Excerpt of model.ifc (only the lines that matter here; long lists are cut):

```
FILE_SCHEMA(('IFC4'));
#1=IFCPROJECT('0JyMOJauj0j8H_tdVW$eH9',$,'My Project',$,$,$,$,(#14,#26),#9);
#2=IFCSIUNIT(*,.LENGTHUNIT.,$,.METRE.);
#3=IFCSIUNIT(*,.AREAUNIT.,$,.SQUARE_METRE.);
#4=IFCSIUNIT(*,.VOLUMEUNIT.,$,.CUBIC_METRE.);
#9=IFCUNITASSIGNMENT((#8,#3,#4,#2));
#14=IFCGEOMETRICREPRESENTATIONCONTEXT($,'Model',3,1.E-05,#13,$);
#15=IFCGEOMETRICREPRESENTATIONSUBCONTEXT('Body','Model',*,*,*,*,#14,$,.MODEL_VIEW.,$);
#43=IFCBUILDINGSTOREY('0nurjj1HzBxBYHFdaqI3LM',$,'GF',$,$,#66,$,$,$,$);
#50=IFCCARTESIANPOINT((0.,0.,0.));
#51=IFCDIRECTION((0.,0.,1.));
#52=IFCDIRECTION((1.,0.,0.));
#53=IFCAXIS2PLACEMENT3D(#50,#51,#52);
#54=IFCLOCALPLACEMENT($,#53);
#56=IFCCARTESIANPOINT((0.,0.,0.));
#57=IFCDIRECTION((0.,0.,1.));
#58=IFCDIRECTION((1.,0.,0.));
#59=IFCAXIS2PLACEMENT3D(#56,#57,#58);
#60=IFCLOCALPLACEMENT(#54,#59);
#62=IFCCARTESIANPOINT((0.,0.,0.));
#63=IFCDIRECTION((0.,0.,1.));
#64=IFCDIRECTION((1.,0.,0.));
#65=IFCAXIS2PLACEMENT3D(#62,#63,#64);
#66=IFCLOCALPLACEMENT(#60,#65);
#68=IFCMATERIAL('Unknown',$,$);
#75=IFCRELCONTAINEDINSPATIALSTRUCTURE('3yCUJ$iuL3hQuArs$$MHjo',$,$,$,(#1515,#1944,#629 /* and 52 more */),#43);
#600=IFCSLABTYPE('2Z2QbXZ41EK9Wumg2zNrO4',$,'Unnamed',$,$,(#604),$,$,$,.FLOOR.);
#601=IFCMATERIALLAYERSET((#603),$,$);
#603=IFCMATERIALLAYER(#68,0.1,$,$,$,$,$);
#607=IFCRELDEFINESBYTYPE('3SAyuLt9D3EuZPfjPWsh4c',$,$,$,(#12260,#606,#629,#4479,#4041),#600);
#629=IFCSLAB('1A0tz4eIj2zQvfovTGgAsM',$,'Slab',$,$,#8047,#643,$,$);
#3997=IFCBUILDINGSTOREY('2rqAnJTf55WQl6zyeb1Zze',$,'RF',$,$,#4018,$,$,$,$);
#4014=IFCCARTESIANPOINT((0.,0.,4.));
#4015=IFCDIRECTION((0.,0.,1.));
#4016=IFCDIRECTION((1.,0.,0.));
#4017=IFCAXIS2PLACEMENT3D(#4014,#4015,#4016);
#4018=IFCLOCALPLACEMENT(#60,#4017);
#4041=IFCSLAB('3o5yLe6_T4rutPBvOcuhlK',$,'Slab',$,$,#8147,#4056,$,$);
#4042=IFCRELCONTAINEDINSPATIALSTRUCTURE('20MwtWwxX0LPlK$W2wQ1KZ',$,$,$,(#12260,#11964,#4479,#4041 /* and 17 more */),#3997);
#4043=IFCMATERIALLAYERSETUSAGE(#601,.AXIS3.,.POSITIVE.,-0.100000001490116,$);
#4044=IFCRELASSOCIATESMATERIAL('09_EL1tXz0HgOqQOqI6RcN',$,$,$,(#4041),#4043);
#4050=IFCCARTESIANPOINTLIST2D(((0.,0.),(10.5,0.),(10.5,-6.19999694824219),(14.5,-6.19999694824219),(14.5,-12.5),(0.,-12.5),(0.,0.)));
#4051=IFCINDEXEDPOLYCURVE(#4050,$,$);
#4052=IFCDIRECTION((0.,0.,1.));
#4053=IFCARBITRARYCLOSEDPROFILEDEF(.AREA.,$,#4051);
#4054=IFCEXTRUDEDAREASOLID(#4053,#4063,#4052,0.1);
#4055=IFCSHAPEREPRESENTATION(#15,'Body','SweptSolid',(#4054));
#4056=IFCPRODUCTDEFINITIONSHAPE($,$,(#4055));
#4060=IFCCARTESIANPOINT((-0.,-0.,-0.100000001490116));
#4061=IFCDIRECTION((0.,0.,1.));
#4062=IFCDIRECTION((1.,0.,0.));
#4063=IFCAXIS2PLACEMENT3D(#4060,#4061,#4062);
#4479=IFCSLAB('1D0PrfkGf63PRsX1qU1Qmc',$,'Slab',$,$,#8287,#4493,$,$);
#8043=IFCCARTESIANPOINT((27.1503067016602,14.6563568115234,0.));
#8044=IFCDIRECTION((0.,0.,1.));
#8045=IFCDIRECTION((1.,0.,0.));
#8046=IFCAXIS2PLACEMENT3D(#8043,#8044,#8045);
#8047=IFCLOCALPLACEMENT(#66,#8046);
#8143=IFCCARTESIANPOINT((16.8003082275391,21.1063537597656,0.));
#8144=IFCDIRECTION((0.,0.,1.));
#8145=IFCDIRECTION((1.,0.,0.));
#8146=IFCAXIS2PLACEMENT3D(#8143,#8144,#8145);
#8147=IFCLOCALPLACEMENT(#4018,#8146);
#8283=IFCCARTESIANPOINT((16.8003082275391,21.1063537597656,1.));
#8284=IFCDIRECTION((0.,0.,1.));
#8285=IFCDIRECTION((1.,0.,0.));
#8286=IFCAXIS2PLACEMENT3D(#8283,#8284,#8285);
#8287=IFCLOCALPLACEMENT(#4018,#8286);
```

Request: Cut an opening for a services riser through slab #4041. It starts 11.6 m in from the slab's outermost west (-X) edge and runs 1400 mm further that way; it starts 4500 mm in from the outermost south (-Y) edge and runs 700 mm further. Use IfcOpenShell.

```python
import numpy as np
import ifcopenshell
import ifcopenshell.api.feature
import ifcopenshell.api.geometry
import ifcopenshell.api.root
import ifcopenshell.geom
import ifcopenshell.util.placement
import ifcopenshell.util.representation
import ifcopenshell.util.shape
import ifcopenshell.util.unit

model = ifcopenshell.open("model.ifc")
unit_scale = ifcopenshell.util.unit.calculate_unit_scale(model)
settings = ifcopenshell.geom.settings()


def volume(element):
    """Net volume in cubic metres, openings subtracted."""
    shape = ifcopenshell.geom.create_shape(settings, element)
    return ifcopenshell.util.shape.get_volume(shape.geometry)


slab = model.by_id(4041)
before = volume(slab)

# Extent in the slab's own axes, in metres. The edges named are its -X and -Y sides.
slab_shape = ifcopenshell.geom.create_shape(settings, slab)
vertices = ifcopenshell.util.shape.get_vertices(slab_shape.geometry)
x_min, y_min, bottom = vertices.min(axis=0)
top = vertices[:, 2].max()

opening = ifcopenshell.api.root.create_entity(model, ifc_class="IfcOpeningElement", name="Services riser opening", predefined_type="OPENING")
context = ifcopenshell.util.representation.get_context(model, "Model", "Body", "MODEL_VIEW")
width, depth = 1.4, 0.7
outline = [(0.0, 0.0), (width, 0.0), (width, depth), (0.0, depth), (0.0, 0.0)]
# Overshoot both faces by 50 mm so the cut is clean.
shape = ifcopenshell.api.geometry.add_slab_representation(
    model, context=context, depth=top - bottom + 0.1, polyline=outline
)
ifcopenshell.api.geometry.assign_representation(model, product=opening, representation=shape)

matrix = ifcopenshell.util.placement.get_local_placement(slab.ObjectPlacement)
matrix[:, 3] = matrix @ np.append(np.array([x_min + 11.6, y_min + 4.5, bottom - 0.05]) / unit_scale, 1.0)
ifcopenshell.api.geometry.edit_object_placement(model, product=opening, matrix=matrix, is_si=False)
ifcopenshell.api.feature.add_feature(model, feature=opening, element=slab)

after = volume(slab)

print(f"slab volume {before:.3f} -> {after:.3f} m3")

model.write("model_edited.ifc")
```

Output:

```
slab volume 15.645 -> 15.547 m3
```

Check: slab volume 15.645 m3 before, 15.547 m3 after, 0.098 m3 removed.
